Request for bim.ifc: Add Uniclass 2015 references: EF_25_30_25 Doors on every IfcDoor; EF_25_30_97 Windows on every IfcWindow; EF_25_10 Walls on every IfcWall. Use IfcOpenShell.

First a look at what the model holds.

```python
import ifcopenshell

model = ifcopenshell.open("bim.ifc")
print(model.schema)
print("classifications:", [c.Name for c in model.by_type("IfcClassification")])
for ifc_class in ("IfcDoor", "IfcRoof", "IfcStair", "IfcWall", "IfcWindow"):
    print(ifc_class, len(model.by_type(ifc_class)))
```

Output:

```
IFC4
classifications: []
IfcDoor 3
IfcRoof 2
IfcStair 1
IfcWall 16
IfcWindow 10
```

```python
import ifcopenshell
import ifcopenshell.api.classification

model = ifcopenshell.open("bim.ifc")

system = ifcopenshell.api.classification.add_classification(model, classification="Uniclass 2015")

codes = {
    "IfcDoor": ("EF_25_30_25", "Doors"),
    "IfcWindow": ("EF_25_30_97", "Windows"),
    "IfcWall": ("EF_25_10", "Walls"),
}
for ifc_class, (code, name) in codes.items():
    products = model.by_type(ifc_class)
    ifcopenshell.api.classification.add_reference(
        model, products=products, classification=system, identification=code, name=name
    )
    print(code, len(products))

model.write("bim_edited.ifc")
```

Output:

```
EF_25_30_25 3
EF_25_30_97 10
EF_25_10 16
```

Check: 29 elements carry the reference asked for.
